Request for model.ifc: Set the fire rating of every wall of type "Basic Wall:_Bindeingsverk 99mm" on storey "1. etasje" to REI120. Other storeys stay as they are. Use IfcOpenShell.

First a look at what the model holds.

```python
import ifcopenshell
import ifcopenshell.util.element

model = ifcopenshell.open("model.ifc")
print(model.schema)
storey = next(s for s in model.by_type("IfcBuildingStorey") if s.Name == "1. etasje")
walls = [e for e in ifcopenshell.util.element.get_decomposition(storey) if e.is_a("IfcWall")]
seen = {}
for e in walls:
    element_type = ifcopenshell.util.element.get_type(e)
    key = (element_type.Name if element_type != e and element_type else None, ifcopenshell.util.element.get_pset(e, "Pset_WallCommon", "FireRating"))
    seen[key] = seen.get(key, 0) + 1
for (name, value), count in sorted(seen.items(), key=str):
    print(count, "x", name, "|", value)
```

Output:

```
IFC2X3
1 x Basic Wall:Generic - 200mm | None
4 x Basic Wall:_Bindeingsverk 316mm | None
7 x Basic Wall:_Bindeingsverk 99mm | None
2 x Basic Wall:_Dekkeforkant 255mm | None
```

```python
import ifcopenshell
import ifcopenshell.api.pset
import ifcopenshell.util.element

model = ifcopenshell.open("model.ifc")

storey = next(s for s in model.by_type("IfcBuildingStorey") if s.Name == "1. etasje")
walls = [e for e in ifcopenshell.util.element.get_decomposition(storey) if e.is_a("IfcWall")]

count = 0
for e in walls:
    element_type = ifcopenshell.util.element.get_type(e)
    if element_type in (None, e) or element_type.Name != "Basic Wall:_Bindeingsverk 99mm":
        continue
    # add_pset returns the element's existing set when there is one.
    pset = ifcopenshell.api.pset.add_pset(model, product=e, name="Pset_WallCommon")
    ifcopenshell.api.pset.edit_pset(model, pset=pset, properties={"FireRating": "REI120"})
    count += 1

print(count, "walls updated")

model.write("model_edited.ifc")
```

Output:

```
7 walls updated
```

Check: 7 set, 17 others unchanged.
